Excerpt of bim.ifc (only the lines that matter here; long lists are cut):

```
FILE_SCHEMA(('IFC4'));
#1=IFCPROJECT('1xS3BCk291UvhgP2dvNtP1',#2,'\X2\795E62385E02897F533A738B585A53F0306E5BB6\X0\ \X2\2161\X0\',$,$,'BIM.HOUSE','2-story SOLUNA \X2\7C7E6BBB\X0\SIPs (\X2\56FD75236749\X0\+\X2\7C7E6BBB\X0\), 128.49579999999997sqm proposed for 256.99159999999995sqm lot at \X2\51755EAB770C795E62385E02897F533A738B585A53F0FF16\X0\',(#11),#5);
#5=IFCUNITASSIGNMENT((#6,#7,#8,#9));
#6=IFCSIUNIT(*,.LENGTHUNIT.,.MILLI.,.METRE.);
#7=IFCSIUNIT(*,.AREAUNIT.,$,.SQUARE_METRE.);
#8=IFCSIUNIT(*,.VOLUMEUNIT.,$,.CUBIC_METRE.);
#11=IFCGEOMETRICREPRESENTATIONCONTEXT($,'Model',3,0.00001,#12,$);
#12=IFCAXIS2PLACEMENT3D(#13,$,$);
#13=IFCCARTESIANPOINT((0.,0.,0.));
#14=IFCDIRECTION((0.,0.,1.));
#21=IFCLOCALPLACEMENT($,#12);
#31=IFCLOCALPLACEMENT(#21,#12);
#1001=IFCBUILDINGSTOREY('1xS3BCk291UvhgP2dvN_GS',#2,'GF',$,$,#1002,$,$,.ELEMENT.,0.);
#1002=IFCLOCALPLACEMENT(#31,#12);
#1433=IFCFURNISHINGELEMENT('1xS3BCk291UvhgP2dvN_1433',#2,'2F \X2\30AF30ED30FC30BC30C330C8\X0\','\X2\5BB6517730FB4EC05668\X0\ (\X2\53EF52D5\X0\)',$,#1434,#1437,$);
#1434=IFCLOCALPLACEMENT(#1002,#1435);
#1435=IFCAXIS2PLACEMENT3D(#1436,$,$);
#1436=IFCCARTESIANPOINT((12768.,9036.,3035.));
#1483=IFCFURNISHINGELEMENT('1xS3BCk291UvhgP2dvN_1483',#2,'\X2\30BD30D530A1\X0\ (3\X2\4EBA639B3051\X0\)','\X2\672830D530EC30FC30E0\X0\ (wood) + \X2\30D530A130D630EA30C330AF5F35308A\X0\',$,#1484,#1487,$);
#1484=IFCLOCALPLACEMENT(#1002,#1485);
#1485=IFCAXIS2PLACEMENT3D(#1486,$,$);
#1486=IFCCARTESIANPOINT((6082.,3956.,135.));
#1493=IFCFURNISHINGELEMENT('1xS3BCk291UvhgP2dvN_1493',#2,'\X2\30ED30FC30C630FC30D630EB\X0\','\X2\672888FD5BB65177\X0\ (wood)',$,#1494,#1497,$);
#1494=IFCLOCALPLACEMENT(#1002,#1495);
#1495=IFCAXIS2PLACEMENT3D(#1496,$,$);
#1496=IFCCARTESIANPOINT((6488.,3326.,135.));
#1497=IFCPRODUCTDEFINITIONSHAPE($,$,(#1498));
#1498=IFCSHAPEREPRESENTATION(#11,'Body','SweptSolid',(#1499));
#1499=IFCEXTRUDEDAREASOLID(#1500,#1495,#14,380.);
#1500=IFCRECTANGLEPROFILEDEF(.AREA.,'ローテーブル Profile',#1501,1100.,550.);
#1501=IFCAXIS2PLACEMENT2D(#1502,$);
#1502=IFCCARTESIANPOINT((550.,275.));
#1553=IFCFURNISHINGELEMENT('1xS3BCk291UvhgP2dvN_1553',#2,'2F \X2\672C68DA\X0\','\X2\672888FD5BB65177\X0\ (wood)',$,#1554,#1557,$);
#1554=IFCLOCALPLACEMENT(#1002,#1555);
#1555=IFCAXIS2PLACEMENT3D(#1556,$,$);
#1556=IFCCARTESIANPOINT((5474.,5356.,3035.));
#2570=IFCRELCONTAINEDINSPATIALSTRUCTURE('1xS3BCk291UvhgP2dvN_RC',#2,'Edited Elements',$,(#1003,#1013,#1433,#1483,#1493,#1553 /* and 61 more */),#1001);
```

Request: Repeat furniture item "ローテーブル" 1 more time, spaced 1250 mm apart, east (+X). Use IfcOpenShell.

```python
import numpy as np
import ifcopenshell
import ifcopenshell.api.geometry
import ifcopenshell.api.root
import ifcopenshell.util.element
import ifcopenshell.util.placement
import ifcopenshell.util.unit

model = ifcopenshell.open("bim.ifc")
unit_scale = ifcopenshell.util.unit.calculate_unit_scale(model)


def reuse_history(source, copy):
    """copy_class also copies each property set's owner history, people and application; keep the originals."""
    for rel in copy.IsDefinedBy:
        if rel.is_a("IfcRelDefinesByProperties") and (history := rel.RelatingPropertyDefinition.OwnerHistory):
            rel.RelatingPropertyDefinition.OwnerHistory = source.OwnerHistory
            ifcopenshell.util.element.remove_deep2(model, history)


source = model.by_guid("1xS3BCk291UvhgP2dvN_1493")
base = ifcopenshell.util.placement.get_local_placement(source.ObjectPlacement)
step = np.array([1.0, 0.0, 0.0]) * 1.25 / unit_scale

for i in range(1, 2):
    copy = ifcopenshell.api.root.copy_class(model, product=source)
    copy.Representation = ifcopenshell.util.element.copy_deep(
        model, source.Representation, exclude=["IfcGeometricRepresentationContext", "IfcRepresentationMap"]
    )
    reuse_history(source, copy)
    matrix = base.copy()
    matrix[:3, 3] += i * step
    print("added at", matrix[:3, 3].round(3) + 0.0)
    ifcopenshell.api.geometry.edit_object_placement(model, product=copy, matrix=matrix, is_si=False)

model.write("bim-out.ifc")
```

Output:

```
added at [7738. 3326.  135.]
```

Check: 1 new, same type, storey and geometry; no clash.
